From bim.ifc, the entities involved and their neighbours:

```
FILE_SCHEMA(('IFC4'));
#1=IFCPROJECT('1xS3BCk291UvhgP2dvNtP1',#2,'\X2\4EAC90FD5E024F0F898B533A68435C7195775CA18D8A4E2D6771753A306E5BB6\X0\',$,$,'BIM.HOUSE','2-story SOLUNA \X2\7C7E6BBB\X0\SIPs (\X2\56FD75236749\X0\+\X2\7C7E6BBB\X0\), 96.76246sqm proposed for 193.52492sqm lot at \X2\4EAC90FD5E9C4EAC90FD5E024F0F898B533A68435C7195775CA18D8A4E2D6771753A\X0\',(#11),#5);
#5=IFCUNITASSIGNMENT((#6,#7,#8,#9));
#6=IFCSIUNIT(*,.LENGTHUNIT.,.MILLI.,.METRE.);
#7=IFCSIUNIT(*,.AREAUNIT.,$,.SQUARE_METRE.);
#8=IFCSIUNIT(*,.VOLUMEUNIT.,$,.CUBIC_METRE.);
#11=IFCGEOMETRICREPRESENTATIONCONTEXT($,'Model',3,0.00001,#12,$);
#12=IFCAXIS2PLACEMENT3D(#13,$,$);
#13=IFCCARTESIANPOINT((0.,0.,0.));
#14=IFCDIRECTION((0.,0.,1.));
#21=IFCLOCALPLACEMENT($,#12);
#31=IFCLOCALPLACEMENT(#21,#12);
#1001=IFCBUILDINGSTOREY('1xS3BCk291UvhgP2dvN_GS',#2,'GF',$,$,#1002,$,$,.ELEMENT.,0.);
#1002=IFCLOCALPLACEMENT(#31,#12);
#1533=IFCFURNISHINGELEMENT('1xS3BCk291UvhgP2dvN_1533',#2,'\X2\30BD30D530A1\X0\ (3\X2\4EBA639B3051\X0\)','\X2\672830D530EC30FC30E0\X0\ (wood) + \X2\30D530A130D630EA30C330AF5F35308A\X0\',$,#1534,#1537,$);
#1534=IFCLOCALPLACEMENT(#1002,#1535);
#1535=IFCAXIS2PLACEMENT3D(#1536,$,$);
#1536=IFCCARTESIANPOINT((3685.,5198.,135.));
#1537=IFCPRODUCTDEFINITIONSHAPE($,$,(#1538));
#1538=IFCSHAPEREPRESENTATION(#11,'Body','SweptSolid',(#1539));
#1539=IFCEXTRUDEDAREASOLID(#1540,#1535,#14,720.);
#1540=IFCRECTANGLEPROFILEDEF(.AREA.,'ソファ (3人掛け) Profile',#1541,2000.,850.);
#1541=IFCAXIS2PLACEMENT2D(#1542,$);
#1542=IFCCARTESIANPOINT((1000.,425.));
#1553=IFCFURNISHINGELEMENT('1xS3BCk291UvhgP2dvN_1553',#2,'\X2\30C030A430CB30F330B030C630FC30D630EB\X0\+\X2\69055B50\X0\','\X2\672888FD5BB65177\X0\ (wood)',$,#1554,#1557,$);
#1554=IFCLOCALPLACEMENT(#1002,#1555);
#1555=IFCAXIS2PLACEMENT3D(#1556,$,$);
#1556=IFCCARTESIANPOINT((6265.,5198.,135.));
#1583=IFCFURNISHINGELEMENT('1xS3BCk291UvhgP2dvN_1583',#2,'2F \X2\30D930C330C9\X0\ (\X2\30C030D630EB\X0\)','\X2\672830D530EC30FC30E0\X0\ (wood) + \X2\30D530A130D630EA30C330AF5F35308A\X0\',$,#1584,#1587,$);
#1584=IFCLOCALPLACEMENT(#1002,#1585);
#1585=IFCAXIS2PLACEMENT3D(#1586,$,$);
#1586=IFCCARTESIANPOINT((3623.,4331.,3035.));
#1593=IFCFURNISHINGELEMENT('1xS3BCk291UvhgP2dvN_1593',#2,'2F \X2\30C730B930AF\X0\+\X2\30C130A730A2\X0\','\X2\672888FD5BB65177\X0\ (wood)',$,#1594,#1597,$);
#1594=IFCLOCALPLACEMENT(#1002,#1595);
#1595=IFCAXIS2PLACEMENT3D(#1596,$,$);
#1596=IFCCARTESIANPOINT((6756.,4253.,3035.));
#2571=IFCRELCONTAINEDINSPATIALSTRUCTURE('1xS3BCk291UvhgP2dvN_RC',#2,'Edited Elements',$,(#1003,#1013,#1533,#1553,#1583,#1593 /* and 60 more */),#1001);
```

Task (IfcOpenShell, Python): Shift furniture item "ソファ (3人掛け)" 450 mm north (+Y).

```python
import ifcopenshell
import ifcopenshell.api.geometry
import ifcopenshell.util.placement
import ifcopenshell.util.unit

model = ifcopenshell.open("bim.ifc")
unit_scale = ifcopenshell.util.unit.calculate_unit_scale(model)

item = model.by_guid("1xS3BCk291UvhgP2dvN_1533")
matrix = ifcopenshell.util.placement.get_local_placement(item.ObjectPlacement)
matrix[1, 3] += 0.45 / unit_scale
ifcopenshell.api.geometry.edit_object_placement(model, product=item, matrix=matrix, is_si=False)

print(ifcopenshell.util.placement.get_local_placement(item.ObjectPlacement).round(3) + 0.0)

model.write("bim-out.ifc")
```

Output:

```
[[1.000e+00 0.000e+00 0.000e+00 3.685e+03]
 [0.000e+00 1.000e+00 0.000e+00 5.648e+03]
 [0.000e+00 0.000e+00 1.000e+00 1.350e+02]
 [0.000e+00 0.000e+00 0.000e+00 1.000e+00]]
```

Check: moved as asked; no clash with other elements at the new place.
